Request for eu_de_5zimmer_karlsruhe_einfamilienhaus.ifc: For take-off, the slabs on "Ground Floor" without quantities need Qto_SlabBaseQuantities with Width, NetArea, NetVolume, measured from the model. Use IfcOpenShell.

First a look at what the model holds.

```python
import ifcopenshell
import ifcopenshell.util.element
import ifcopenshell.util.unit

model = ifcopenshell.open("eu_de_5zimmer_karlsruhe_einfamilienhaus.ifc")
print(model.schema)
for unit_type in ("LENGTHUNIT", "AREAUNIT", "VOLUMEUNIT"):
    print(unit_type, ifcopenshell.util.unit.calculate_unit_scale(model, unit_type))
storey = next(s for s in model.by_type("IfcBuildingStorey") if s.Name == "Ground Floor")
slabs = [e for e in ifcopenshell.util.element.get_decomposition(storey) if e.is_a("IfcSlab")]
for e in sorted(slabs, key=lambda e: e.id()):
    print(e.id(), e.is_a(), e.Name, list(ifcopenshell.util.element.get_psets(e, qtos_only=True)), sep=" | ")
```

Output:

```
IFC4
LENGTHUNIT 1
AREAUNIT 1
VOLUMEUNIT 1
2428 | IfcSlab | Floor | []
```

```python
import ifcopenshell
import ifcopenshell.api.pset
import ifcopenshell.geom
import ifcopenshell.util.element
import ifcopenshell.util.shape
import ifcopenshell.util.unit

model = ifcopenshell.open("eu_de_5zimmer_karlsruhe_einfamilienhaus.ifc")
unit_scale = ifcopenshell.util.unit.calculate_unit_scale(model)
area_scale = ifcopenshell.util.unit.calculate_unit_scale(model, "AREAUNIT")
volume_scale = ifcopenshell.util.unit.calculate_unit_scale(model, "VOLUMEUNIT")
settings = ifcopenshell.geom.settings()

storey = next(s for s in model.by_type("IfcBuildingStorey") if s.Name == "Ground Floor")
slabs = [e for e in ifcopenshell.util.element.get_decomposition(storey) if e.is_a("IfcSlab")]

for e in sorted(slabs, key=lambda e: e.id()):
    if ifcopenshell.util.element.get_psets(e, qtos_only=True, should_inherit=False):
        continue
    # Geometry comes back in metres, in the element's own axes.
    shape = ifcopenshell.geom.create_shape(settings, e)
    values = {
        "Width": ifcopenshell.util.shape.get_z(shape.geometry) / unit_scale,
        "NetArea": ifcopenshell.util.shape.get_footprint_area(shape.geometry) / area_scale,
        "NetVolume": ifcopenshell.util.shape.get_volume(shape.geometry) / volume_scale,
    }
    qto = ifcopenshell.api.pset.add_qto(model, product=e, name="Qto_SlabBaseQuantities")
    ifcopenshell.api.pset.edit_qto(model, qto=qto, properties=values)
    print(e.id(), {k: round(v, 3) for k, v in values.items()})

model.write("eu_de_5zimmer_karlsruhe_einfamilienhaus_edited.ifc")
```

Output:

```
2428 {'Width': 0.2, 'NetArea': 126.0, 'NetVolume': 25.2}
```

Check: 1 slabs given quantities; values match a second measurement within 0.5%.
